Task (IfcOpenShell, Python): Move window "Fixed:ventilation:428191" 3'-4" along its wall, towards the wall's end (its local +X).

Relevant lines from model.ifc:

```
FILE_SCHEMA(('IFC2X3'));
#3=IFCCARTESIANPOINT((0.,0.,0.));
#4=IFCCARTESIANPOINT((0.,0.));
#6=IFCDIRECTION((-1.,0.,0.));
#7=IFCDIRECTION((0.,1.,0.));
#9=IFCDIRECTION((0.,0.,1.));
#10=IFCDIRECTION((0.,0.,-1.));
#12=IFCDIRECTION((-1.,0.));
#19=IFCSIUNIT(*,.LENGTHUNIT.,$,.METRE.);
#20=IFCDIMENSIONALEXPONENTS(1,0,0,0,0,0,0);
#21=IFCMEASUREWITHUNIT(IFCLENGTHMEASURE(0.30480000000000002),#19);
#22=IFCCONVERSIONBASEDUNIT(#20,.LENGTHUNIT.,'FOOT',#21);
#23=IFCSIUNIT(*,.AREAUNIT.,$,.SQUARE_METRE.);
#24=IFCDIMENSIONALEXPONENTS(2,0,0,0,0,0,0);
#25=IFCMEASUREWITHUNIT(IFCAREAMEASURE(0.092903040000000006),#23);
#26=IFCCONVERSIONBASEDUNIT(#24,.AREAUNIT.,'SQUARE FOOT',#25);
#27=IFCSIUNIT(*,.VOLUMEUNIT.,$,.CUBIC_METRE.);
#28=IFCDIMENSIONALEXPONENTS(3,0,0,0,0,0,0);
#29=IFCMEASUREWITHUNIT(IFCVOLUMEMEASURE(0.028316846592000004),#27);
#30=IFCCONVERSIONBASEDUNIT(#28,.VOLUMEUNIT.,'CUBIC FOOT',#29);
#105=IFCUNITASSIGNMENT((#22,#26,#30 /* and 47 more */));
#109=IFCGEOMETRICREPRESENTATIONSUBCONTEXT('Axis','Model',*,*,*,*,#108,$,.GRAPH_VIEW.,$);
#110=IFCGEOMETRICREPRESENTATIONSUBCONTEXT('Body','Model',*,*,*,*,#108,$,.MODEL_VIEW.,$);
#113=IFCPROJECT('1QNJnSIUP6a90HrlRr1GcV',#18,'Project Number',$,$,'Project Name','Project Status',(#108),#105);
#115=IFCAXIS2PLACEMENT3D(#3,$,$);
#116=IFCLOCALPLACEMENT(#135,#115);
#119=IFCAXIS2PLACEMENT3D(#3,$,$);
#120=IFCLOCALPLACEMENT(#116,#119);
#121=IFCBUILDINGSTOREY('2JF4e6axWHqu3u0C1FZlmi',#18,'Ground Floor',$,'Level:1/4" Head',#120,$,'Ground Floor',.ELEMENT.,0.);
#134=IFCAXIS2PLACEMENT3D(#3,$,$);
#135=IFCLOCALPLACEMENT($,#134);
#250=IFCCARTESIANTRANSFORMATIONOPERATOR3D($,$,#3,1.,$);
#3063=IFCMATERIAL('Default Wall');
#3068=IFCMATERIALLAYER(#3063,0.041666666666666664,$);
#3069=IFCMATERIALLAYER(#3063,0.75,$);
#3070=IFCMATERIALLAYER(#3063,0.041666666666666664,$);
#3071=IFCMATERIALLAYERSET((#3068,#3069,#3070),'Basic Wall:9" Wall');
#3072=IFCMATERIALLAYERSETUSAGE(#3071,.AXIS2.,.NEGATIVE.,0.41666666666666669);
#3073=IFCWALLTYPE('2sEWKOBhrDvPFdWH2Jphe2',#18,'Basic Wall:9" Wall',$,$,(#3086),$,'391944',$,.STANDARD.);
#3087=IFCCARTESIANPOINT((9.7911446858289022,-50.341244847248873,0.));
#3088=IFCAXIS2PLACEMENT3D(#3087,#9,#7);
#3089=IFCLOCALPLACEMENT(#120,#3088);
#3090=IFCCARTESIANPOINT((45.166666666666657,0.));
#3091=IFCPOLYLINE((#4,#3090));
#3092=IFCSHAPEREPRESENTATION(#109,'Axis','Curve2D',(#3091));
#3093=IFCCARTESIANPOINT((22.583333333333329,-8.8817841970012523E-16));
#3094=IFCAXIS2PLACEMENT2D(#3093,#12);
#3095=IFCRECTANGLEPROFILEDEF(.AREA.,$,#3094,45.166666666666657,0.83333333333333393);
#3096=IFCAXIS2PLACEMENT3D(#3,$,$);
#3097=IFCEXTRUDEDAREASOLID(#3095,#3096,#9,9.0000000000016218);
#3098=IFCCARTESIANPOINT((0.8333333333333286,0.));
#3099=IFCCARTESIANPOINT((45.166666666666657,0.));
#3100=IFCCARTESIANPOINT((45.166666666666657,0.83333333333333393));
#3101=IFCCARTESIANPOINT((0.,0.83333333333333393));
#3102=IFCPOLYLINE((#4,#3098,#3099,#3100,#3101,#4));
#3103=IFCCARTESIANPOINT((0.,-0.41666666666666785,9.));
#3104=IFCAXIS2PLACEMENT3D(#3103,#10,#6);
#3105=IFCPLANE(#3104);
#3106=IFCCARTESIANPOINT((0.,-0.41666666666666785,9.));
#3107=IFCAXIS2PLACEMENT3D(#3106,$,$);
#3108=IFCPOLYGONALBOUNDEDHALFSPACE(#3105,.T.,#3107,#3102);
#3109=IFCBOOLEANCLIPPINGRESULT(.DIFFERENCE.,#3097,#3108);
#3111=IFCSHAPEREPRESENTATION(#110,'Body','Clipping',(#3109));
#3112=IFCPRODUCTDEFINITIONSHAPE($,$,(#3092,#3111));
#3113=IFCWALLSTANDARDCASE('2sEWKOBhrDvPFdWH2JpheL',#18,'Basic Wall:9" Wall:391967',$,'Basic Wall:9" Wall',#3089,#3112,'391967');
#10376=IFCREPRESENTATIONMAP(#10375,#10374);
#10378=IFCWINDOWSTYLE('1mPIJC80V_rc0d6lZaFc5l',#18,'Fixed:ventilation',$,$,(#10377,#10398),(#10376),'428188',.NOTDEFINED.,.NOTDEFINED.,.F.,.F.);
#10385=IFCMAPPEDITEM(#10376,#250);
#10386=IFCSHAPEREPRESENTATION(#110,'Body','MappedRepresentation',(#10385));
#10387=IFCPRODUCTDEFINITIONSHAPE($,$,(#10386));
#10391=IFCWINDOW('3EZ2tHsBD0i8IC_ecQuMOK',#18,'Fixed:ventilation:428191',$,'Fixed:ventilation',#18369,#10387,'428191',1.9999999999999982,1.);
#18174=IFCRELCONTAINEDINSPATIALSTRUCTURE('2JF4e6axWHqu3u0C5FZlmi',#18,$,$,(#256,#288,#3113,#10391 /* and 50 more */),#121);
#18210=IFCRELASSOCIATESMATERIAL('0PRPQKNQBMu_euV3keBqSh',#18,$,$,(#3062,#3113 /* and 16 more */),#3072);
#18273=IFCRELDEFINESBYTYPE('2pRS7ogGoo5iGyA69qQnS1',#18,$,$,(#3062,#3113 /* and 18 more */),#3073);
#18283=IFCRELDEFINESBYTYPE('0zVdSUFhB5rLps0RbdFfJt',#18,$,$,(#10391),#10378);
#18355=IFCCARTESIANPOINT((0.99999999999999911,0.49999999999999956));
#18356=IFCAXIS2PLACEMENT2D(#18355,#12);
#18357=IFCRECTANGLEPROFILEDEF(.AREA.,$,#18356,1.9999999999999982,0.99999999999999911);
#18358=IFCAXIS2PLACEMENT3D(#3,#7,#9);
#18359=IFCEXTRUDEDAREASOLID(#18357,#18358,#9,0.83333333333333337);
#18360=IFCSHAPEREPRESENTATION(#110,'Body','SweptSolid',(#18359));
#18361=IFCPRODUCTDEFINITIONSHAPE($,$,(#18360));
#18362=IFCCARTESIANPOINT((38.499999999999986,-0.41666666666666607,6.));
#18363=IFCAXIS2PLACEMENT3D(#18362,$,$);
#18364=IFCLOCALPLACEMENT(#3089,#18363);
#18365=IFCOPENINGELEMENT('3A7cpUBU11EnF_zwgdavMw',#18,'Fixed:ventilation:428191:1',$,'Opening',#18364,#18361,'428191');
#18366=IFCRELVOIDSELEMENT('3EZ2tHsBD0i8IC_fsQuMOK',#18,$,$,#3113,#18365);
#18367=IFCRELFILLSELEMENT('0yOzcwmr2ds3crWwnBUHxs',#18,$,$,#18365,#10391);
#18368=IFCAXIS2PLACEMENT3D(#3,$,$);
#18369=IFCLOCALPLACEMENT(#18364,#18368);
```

```python
import ifcopenshell
import ifcopenshell.api.geometry
import ifcopenshell.util.placement
import ifcopenshell.util.unit

model = ifcopenshell.open("model.ifc")
unit_scale = ifcopenshell.util.unit.calculate_unit_scale(model)

window = model.by_guid("3EZ2tHsBD0i8IC_ecQuMOK")
opening = window.FillsVoids[0].RelatingOpeningElement
wall = opening.VoidsElements[0].RelatingBuildingElement

wall_matrix = ifcopenshell.util.placement.get_local_placement(wall.ObjectPlacement)
shift = wall_matrix[:3, 0] * 40 * 0.0254 / unit_scale
before = ifcopenshell.util.placement.get_local_placement(window.ObjectPlacement)[:3, 3].copy()

# The window is placed relative to its opening, so it follows when the opening moves.
matrix = ifcopenshell.util.placement.get_local_placement(opening.ObjectPlacement)
matrix[:3, 3] += shift
ifcopenshell.api.geometry.edit_object_placement(
    model, product=opening, matrix=matrix, is_si=False, should_transform_children=True
)

after = ifcopenshell.util.placement.get_local_placement(window.ObjectPlacement)[:3, 3]
print("window moved by", (after - before).round(3) + 0.0)

model.write("model_updated.ifc")
```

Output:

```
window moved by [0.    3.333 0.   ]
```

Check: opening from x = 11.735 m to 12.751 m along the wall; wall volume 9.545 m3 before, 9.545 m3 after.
